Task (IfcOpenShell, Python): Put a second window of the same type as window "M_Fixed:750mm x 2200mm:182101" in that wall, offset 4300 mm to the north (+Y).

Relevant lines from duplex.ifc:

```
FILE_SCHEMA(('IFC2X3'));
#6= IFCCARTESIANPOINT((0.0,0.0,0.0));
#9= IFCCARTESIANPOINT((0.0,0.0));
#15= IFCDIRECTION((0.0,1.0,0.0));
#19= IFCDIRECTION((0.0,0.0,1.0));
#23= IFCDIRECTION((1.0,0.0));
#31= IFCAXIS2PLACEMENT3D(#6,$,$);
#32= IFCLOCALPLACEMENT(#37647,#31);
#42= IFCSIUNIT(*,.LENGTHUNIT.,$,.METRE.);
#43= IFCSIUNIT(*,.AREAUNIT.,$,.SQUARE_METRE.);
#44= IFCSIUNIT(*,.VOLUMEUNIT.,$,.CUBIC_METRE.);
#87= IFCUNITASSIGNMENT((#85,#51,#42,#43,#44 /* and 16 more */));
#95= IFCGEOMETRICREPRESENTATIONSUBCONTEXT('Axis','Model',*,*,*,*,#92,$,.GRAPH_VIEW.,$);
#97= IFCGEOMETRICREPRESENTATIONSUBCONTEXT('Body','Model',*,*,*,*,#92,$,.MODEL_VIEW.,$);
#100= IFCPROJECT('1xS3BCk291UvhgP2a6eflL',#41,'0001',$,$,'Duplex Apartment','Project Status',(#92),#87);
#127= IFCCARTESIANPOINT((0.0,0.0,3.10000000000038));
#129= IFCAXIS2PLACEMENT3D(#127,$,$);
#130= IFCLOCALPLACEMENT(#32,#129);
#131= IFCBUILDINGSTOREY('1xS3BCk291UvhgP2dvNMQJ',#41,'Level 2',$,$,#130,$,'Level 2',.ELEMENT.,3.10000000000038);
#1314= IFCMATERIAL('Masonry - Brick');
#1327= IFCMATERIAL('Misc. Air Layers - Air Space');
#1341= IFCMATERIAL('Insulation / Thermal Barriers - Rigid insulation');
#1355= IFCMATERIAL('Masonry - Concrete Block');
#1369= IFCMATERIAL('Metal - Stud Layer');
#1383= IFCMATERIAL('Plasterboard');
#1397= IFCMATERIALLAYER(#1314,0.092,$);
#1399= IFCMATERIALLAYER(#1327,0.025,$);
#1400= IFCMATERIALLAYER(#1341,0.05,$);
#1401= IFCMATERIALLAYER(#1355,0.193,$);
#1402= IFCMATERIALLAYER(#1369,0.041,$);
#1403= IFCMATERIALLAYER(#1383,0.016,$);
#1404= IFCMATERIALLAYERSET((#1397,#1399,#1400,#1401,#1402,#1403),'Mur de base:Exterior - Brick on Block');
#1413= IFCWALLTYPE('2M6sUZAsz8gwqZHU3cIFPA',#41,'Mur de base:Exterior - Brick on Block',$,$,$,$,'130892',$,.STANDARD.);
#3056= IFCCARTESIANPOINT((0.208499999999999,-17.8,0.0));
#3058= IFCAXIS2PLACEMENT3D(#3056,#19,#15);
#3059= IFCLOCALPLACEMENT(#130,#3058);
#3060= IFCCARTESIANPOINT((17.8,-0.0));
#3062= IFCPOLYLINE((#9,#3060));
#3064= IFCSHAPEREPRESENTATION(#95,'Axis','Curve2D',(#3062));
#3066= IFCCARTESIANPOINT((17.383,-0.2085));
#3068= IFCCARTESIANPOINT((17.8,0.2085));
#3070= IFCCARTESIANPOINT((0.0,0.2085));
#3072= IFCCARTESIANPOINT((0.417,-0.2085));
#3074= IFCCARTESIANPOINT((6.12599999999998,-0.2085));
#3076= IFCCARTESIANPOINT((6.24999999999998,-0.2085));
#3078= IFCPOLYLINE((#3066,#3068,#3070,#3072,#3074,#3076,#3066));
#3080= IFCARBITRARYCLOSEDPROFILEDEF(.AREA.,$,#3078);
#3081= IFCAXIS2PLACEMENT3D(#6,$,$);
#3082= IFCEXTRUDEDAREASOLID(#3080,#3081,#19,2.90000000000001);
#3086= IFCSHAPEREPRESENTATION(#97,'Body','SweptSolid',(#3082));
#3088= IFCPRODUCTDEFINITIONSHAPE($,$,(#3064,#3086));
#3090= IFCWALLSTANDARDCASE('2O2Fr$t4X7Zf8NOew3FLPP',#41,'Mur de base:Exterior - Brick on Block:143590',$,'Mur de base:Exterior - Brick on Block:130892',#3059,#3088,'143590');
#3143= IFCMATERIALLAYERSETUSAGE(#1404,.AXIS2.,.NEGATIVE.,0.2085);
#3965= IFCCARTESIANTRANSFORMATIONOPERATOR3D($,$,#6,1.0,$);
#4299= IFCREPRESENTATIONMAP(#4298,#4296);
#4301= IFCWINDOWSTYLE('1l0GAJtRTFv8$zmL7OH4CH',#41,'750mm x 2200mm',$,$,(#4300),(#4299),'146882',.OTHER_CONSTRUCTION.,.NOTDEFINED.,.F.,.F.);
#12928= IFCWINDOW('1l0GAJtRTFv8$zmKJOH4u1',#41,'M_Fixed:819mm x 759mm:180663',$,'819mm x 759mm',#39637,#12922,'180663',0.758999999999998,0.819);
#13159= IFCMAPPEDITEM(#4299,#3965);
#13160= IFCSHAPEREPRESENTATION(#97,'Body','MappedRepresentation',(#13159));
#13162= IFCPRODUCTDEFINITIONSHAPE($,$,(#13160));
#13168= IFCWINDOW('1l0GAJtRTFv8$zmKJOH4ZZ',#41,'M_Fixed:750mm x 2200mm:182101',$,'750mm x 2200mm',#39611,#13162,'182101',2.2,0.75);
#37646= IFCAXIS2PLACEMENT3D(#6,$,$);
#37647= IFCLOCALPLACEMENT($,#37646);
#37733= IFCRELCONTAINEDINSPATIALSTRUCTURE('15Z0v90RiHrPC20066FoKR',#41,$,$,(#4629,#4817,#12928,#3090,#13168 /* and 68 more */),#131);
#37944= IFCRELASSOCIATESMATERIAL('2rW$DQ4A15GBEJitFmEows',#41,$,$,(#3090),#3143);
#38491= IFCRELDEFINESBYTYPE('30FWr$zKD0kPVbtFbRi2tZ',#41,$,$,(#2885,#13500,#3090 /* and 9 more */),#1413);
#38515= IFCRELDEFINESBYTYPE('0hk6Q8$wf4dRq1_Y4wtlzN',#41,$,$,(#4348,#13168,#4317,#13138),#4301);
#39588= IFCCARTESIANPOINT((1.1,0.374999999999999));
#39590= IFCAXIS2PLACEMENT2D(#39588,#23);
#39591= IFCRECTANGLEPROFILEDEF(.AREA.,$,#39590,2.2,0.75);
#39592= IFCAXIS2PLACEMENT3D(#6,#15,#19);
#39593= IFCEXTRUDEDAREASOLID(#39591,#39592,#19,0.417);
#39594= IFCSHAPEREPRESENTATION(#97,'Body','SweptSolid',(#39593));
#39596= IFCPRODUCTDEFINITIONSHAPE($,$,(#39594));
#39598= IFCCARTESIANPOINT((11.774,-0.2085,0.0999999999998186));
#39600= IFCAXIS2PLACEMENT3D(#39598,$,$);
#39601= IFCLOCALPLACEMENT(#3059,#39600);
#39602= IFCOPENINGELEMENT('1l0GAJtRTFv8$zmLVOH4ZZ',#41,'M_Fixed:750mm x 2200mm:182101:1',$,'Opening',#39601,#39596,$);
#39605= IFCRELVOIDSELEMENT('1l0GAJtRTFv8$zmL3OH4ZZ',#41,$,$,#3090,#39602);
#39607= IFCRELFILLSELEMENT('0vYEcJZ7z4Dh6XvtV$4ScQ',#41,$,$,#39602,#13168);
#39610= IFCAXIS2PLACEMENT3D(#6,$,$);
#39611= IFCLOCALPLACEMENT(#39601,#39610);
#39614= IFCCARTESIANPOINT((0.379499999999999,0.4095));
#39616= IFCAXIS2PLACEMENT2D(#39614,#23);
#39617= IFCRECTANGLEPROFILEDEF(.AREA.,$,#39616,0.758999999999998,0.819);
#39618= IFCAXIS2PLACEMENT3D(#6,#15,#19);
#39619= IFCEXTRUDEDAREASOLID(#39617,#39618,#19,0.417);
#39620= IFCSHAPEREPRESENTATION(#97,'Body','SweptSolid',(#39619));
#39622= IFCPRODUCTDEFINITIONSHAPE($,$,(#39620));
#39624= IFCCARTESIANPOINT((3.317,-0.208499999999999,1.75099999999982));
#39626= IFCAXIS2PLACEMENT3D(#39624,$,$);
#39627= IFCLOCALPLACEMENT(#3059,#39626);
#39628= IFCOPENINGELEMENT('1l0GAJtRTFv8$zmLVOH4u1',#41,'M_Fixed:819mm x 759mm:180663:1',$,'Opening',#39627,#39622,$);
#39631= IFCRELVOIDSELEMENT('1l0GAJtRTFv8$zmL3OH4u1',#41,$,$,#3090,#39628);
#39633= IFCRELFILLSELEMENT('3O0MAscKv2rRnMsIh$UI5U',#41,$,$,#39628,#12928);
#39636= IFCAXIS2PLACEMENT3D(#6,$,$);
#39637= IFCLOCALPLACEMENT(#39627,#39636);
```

```python
import ifcopenshell
import ifcopenshell.api.feature
import ifcopenshell.api.geometry
import ifcopenshell.api.root
import ifcopenshell.geom
import ifcopenshell.util.element
import ifcopenshell.util.placement
import ifcopenshell.util.shape
import ifcopenshell.util.unit

model = ifcopenshell.open("duplex.ifc")
unit_scale = ifcopenshell.util.unit.calculate_unit_scale(model)
settings = ifcopenshell.geom.settings()


def volume(element):
    """Net volume in cubic metres, openings subtracted."""
    shape = ifcopenshell.geom.create_shape(settings, element)
    return ifcopenshell.util.shape.get_volume(shape.geometry)


def reuse_history(source, copy):
    """copy_class also copies each property set's owner history, people and application; keep the originals."""
    for rel in copy.IsDefinedBy:
        if rel.is_a("IfcRelDefinesByProperties") and (history := rel.RelatingPropertyDefinition.OwnerHistory):
            rel.RelatingPropertyDefinition.OwnerHistory = source.OwnerHistory
            ifcopenshell.util.element.remove_deep2(model, history)


window = model.by_id(13168)
opening = window.FillsVoids[0].RelatingOpeningElement
wall = opening.VoidsElements[0].RelatingBuildingElement
before = volume(wall)
shift = ifcopenshell.util.placement.get_local_placement(wall.ObjectPlacement)[:3, 0] * 4.3 / unit_scale

# copy_class copies the void relationship, type, container and properties, but no geometry.
new_opening = ifcopenshell.api.root.copy_class(model, product=opening)
new_opening.Representation = ifcopenshell.util.element.copy_deep(
    model, opening.Representation, exclude=["IfcGeometricRepresentationContext", "IfcRepresentationMap"]
)
new_opening.Name = "M_Fixed:750mm x 2200mm"
new_window = ifcopenshell.api.root.copy_class(model, product=window)
new_window.Representation = ifcopenshell.util.element.copy_deep(
    model, window.Representation, exclude=["IfcGeometricRepresentationContext", "IfcRepresentationMap"]
)
new_window.Name = "M_Fixed:750mm x 2200mm"
new_window.Tag = None
reuse_history(window, new_window)
fills = ifcopenshell.api.feature.add_filling(model, opening=new_opening, element=new_window)
fills.OwnerHistory = new_window.OwnerHistory  # required in IFC2X3

for old, new in ((opening, new_opening), (window, new_window)):
    matrix = ifcopenshell.util.placement.get_local_placement(old.ObjectPlacement)
    matrix[:3, 3] += shift
    ifcopenshell.api.geometry.edit_object_placement(model, product=new, matrix=matrix, is_si=False)

after = volume(wall)

print(f"wall volume {before:.3f} -> {after:.3f} m3")

model.write("duplex_updated.ifc")
```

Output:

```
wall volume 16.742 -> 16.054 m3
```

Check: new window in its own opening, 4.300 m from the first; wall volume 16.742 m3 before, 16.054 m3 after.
